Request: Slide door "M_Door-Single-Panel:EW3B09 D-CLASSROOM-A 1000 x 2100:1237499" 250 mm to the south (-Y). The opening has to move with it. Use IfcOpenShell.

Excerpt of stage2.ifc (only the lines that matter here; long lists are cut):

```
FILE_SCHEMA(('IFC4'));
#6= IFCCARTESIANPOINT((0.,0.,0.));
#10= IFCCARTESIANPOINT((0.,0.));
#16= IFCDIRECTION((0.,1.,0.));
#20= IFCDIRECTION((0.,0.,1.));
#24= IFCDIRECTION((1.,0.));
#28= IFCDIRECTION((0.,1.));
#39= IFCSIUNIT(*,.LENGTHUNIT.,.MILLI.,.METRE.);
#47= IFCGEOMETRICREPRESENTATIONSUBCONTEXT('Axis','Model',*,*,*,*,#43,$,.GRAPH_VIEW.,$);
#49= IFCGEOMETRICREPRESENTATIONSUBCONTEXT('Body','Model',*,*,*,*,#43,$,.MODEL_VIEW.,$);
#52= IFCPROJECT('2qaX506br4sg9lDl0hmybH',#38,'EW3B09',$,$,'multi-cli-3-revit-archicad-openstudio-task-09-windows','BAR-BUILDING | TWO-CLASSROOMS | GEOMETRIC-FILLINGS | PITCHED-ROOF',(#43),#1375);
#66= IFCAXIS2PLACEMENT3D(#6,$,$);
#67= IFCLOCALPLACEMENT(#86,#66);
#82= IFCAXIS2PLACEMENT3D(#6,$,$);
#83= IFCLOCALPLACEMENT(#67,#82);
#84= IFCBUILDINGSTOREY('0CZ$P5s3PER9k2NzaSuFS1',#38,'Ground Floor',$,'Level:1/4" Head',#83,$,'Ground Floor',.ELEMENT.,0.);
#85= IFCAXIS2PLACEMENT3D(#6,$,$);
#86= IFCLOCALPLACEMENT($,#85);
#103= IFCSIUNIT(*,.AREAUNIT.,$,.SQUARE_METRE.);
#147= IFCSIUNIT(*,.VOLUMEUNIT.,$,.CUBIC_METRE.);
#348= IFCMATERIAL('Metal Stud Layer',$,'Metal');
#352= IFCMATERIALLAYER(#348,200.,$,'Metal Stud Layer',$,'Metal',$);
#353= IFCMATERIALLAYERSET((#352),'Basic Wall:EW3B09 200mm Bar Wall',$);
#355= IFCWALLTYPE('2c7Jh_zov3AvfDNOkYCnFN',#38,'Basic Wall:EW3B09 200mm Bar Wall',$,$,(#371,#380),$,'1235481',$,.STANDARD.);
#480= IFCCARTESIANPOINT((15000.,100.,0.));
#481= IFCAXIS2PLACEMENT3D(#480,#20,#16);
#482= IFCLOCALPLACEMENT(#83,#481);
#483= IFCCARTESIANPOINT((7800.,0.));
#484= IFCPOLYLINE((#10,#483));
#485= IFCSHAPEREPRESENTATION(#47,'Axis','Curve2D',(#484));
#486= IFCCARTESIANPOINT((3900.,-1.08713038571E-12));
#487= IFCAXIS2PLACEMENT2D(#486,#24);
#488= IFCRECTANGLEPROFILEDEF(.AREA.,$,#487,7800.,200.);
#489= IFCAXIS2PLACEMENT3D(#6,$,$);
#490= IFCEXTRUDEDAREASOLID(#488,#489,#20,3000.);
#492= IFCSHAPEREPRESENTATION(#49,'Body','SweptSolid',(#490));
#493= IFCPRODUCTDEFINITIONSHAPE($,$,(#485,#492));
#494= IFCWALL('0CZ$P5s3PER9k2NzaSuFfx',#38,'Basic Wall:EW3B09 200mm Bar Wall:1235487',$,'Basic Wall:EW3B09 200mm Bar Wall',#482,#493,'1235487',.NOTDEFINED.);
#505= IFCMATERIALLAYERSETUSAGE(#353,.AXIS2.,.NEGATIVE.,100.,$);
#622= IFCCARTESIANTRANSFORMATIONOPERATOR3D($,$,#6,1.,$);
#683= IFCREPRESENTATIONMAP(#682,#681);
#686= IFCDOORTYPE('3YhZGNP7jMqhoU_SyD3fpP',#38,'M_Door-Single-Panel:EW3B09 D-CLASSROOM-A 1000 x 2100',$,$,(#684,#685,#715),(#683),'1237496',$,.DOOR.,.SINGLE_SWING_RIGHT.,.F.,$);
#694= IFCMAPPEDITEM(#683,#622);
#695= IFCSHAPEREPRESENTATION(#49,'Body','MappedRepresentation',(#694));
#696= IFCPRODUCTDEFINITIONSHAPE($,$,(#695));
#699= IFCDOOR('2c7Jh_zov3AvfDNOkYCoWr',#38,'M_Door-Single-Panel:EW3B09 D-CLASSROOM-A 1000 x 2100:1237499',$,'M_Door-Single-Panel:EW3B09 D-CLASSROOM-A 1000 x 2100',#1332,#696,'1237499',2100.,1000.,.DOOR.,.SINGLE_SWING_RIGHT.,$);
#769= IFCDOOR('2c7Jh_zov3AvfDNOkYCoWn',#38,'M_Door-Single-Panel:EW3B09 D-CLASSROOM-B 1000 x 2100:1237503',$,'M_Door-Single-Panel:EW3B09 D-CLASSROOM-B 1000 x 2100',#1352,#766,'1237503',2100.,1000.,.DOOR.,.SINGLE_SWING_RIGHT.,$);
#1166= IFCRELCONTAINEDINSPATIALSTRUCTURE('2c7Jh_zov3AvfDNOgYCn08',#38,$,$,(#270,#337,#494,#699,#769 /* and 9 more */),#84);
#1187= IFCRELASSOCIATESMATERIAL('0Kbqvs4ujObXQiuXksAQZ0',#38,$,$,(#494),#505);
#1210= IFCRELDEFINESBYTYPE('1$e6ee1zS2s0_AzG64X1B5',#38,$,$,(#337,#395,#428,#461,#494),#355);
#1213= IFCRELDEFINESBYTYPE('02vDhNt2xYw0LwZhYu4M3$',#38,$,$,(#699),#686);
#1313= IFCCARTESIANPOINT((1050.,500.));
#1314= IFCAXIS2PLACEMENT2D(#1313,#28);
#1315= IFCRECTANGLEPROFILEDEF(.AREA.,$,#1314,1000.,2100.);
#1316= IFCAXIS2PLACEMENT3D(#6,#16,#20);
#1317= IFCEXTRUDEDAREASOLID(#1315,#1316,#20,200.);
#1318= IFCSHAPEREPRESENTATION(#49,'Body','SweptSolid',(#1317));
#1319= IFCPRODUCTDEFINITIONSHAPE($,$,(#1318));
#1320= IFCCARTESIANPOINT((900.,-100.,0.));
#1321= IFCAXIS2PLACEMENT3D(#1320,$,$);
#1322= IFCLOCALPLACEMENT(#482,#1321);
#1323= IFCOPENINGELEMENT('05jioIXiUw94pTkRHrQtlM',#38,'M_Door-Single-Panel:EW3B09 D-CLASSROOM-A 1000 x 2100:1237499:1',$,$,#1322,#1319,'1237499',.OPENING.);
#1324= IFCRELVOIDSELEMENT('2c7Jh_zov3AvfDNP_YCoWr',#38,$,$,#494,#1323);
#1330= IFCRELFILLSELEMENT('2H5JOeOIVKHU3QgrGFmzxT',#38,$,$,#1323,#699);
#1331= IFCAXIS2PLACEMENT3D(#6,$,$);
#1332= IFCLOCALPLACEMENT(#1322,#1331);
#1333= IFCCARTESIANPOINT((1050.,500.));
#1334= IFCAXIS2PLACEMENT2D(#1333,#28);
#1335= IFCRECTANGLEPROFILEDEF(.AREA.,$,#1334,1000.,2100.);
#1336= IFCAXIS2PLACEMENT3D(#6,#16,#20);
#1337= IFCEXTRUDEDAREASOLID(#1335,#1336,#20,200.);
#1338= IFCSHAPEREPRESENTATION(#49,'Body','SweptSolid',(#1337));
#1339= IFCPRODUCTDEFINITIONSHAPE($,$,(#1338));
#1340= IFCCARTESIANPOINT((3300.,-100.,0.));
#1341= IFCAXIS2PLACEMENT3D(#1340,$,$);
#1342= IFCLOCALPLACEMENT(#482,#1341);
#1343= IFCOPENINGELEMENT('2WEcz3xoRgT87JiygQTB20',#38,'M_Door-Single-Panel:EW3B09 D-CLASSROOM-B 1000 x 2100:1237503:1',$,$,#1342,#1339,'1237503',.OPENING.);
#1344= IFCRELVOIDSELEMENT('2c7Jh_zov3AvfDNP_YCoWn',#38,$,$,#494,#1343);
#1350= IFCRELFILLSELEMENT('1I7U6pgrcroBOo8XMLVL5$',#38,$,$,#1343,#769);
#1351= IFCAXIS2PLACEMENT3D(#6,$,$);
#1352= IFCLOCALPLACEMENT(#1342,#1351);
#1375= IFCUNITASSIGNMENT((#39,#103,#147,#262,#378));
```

```python
import ifcopenshell
import ifcopenshell.api.geometry
import ifcopenshell.util.placement
import ifcopenshell.util.unit

model = ifcopenshell.open("stage2.ifc")
unit_scale = ifcopenshell.util.unit.calculate_unit_scale(model)

door = model.by_guid("2c7Jh_zov3AvfDNOkYCoWr")
opening = door.FillsVoids[0].RelatingOpeningElement
wall = opening.VoidsElements[0].RelatingBuildingElement

wall_matrix = ifcopenshell.util.placement.get_local_placement(wall.ObjectPlacement)
shift = wall_matrix[:3, 0] * -0.25 / unit_scale
before = ifcopenshell.util.placement.get_local_placement(door.ObjectPlacement)[:3, 3].copy()

# The door is placed relative to its opening, so it follows when the opening moves.
matrix = ifcopenshell.util.placement.get_local_placement(opening.ObjectPlacement)
matrix[:3, 3] += shift
ifcopenshell.api.geometry.edit_object_placement(
    model, product=opening, matrix=matrix, is_si=False, should_transform_children=True
)

after = ifcopenshell.util.placement.get_local_placement(door.ObjectPlacement)[:3, 3]
print("door moved by", (after - before).round(3) + 0.0)

model.write("stage2-out.ifc")
```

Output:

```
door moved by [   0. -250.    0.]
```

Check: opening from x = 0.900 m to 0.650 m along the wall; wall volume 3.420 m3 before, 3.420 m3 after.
